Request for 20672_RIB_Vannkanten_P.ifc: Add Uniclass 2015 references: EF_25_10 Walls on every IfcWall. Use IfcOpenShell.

First a look at what the model holds.

```python
import ifcopenshell

model = ifcopenshell.open("20672_RIB_Vannkanten_P.ifc")
print(model.schema)
print("classifications:", [c.Name for c in model.by_type("IfcClassification")])
for ifc_class in ("IfcDoor", "IfcRoof", "IfcStair", "IfcWall", "IfcWindow"):
    print(ifc_class, len(model.by_type(ifc_class)))
```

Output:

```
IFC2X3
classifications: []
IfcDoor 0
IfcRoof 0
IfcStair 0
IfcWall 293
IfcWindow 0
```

```python
import ifcopenshell
import ifcopenshell.api.classification

model = ifcopenshell.open("20672_RIB_Vannkanten_P.ifc")

# IFC2X3 requires Source and Edition and has no link from the project to the system.
system = model.create_entity("IfcClassification", Source="NBS", Edition="2015", Name="Uniclass 2015")

codes = {
    "IfcWall": ("EF_25_10", "Walls"),
}
for ifc_class, (code, name) in codes.items():
    products = model.by_type(ifc_class)
    ifcopenshell.api.classification.add_reference(
        model, products=products, classification=system, identification=code, name=name
    )
    print(code, len(products))

model.write("20672_RIB_Vannkanten_P_edited.ifc")
```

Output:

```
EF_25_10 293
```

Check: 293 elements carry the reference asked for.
